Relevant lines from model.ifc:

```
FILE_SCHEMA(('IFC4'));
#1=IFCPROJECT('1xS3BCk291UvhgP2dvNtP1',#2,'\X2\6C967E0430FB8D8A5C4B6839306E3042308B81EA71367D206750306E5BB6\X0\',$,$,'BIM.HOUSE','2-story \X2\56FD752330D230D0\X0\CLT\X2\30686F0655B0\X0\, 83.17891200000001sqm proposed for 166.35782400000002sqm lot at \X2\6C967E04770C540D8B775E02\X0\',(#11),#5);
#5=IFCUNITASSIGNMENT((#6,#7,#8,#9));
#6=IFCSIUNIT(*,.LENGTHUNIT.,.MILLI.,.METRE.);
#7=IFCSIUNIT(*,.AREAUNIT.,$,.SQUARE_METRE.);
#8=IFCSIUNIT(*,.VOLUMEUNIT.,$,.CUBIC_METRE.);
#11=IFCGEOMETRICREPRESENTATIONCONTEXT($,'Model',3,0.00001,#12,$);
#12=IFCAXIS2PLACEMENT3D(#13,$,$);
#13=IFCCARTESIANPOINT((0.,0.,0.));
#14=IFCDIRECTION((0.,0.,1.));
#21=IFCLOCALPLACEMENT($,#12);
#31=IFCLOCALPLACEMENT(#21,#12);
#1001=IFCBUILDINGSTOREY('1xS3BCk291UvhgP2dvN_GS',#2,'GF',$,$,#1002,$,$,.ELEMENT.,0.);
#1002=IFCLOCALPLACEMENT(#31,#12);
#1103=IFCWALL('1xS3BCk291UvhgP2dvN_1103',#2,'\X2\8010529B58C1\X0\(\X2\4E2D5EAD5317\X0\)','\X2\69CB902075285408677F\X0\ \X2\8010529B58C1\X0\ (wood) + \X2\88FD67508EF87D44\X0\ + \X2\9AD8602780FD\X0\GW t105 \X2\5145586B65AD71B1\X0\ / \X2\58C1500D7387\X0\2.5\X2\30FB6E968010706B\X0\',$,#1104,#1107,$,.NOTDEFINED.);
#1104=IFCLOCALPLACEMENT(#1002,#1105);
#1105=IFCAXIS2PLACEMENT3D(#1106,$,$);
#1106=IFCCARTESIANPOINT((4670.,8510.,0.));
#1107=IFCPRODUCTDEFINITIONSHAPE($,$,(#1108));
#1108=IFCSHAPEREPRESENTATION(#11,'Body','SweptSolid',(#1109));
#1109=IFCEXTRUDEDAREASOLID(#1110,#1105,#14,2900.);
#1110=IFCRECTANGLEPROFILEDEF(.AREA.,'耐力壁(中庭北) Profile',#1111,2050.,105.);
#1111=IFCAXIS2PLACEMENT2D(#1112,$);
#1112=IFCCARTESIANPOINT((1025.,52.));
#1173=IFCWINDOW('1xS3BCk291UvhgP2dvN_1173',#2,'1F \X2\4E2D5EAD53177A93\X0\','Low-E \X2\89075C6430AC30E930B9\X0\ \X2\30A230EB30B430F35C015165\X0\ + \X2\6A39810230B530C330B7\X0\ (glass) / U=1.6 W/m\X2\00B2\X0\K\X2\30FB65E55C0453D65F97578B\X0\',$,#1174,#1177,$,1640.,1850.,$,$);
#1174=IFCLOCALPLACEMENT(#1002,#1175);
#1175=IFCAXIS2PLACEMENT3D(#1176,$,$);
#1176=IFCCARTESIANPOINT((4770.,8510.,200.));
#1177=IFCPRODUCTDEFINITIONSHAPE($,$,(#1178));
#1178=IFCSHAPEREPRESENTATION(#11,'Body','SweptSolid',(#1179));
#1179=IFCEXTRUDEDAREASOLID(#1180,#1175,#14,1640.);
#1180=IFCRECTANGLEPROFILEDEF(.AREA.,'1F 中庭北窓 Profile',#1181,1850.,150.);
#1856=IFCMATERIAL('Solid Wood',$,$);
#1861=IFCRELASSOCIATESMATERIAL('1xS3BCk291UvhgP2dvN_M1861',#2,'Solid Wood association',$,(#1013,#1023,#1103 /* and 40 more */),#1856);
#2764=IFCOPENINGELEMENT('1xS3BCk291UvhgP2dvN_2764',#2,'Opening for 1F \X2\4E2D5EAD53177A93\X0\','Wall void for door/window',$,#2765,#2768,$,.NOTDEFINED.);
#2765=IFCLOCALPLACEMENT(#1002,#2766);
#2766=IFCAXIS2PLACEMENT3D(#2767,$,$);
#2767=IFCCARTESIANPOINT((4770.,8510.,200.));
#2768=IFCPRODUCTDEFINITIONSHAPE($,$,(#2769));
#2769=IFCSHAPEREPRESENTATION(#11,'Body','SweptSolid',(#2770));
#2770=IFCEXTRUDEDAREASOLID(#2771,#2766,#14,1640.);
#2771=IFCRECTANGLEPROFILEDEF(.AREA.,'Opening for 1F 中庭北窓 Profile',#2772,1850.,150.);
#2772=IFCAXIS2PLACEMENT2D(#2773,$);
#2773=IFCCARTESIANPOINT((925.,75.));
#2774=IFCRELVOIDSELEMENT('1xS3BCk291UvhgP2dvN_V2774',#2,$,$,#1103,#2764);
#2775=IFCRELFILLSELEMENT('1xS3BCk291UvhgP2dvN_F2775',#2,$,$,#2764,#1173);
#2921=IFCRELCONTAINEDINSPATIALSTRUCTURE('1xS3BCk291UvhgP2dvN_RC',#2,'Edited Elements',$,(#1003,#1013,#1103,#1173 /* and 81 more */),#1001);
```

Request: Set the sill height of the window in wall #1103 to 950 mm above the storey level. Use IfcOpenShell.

```python
import numpy as np
import ifcopenshell
import ifcopenshell.api.geometry
import ifcopenshell.geom
import ifcopenshell.util.element
import ifcopenshell.util.placement
import ifcopenshell.util.shape
import ifcopenshell.util.unit

model = ifcopenshell.open("model.ifc")
unit_scale = ifcopenshell.util.unit.calculate_unit_scale(model)

window = model.by_guid("1xS3BCk291UvhgP2dvN_1173")
opening = window.FillsVoids[0].RelatingOpeningElement
storey = ifcopenshell.util.element.get_container(window, ifc_class="IfcBuildingStorey")
level = ifcopenshell.util.placement.get_local_placement(storey.ObjectPlacement)[2, 3]

# The opening's origin need not be at the sill, so measure its lowest point.
shape = ifcopenshell.geom.create_shape(ifcopenshell.geom.settings(), opening)
bottom = ifcopenshell.util.shape.get_shape_bottom_elevation(shape, shape.geometry) / unit_scale
dz = level + 950.0 - bottom

shift = np.array([0.0, 0.0, dz])
# The window is not placed relative to its opening, so move both.
for product in (opening, window):
    matrix = ifcopenshell.util.placement.get_local_placement(product.ObjectPlacement)
    matrix[:3, 3] += shift
    ifcopenshell.api.geometry.edit_object_placement(model, product=product, matrix=matrix, is_si=False)

print(f"moved by {dz * unit_scale:+.3f} m")

model.write("model_updated.ifc")
```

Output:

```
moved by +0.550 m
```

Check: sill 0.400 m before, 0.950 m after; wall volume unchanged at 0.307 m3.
